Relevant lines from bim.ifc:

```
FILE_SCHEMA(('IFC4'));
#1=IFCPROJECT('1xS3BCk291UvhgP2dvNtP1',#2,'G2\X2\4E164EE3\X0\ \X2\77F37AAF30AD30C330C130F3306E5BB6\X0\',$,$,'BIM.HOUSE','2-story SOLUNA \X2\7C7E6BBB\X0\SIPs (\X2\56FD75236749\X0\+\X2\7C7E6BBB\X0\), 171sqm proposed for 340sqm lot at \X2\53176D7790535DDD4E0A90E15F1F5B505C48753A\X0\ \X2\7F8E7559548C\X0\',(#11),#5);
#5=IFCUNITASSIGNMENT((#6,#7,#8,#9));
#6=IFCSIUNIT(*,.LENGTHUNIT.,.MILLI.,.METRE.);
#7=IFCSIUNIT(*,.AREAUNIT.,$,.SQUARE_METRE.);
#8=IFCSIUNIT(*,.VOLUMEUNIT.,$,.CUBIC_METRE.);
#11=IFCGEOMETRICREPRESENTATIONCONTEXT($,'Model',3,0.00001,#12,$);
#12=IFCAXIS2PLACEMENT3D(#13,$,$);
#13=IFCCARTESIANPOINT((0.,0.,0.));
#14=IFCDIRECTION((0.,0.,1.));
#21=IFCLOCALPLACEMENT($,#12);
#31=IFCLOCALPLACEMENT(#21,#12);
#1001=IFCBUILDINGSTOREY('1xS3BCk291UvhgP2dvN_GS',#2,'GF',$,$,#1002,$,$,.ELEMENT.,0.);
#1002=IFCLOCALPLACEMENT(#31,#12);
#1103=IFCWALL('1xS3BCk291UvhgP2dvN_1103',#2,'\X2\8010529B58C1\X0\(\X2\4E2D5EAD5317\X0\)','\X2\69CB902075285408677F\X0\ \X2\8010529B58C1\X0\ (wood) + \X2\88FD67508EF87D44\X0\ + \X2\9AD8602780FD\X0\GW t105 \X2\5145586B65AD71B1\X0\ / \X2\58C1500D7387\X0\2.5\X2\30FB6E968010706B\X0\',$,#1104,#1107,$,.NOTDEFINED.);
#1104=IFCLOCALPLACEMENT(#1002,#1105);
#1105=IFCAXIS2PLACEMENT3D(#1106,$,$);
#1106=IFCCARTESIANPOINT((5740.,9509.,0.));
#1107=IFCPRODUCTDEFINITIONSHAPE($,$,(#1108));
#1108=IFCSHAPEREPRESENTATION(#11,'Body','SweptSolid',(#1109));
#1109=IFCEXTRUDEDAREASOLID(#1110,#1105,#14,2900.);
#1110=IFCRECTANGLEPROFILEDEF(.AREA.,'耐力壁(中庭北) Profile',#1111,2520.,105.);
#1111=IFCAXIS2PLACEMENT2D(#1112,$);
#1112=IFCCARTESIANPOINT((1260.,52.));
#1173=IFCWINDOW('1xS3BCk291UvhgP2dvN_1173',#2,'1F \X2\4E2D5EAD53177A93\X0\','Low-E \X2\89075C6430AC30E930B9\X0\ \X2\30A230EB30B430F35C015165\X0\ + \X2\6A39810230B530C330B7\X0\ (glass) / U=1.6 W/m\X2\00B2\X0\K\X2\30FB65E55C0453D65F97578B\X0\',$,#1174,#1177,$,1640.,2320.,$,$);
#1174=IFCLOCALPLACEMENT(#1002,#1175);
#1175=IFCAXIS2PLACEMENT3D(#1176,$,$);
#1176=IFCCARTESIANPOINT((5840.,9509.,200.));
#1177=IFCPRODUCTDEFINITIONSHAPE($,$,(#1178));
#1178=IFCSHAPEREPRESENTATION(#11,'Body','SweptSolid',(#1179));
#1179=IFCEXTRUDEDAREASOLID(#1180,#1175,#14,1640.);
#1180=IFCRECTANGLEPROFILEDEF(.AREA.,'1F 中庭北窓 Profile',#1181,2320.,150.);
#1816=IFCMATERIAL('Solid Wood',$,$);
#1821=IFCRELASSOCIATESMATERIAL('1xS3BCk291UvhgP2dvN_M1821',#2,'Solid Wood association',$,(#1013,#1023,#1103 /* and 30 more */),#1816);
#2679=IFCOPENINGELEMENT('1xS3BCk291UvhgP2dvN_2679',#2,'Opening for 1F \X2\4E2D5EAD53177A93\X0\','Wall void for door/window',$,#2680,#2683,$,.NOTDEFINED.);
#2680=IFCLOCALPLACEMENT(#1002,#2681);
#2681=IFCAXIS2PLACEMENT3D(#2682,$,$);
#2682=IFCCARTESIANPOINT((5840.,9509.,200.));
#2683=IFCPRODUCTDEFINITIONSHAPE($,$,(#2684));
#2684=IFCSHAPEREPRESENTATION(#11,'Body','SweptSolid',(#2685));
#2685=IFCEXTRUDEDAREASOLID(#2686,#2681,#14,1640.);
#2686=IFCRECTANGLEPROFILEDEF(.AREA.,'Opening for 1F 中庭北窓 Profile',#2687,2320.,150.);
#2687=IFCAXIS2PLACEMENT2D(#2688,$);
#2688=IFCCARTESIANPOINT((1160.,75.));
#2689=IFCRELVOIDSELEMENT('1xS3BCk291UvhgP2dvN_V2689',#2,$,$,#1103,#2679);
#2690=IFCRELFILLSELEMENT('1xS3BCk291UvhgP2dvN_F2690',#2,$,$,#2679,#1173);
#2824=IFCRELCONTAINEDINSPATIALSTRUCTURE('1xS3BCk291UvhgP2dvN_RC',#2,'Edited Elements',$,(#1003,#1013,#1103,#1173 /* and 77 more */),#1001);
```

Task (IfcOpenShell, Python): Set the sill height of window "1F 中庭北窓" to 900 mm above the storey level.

```python
import numpy as np
import ifcopenshell
import ifcopenshell.api.geometry
import ifcopenshell.geom
import ifcopenshell.util.element
import ifcopenshell.util.placement
import ifcopenshell.util.shape
import ifcopenshell.util.unit

model = ifcopenshell.open("bim.ifc")
unit_scale = ifcopenshell.util.unit.calculate_unit_scale(model)

window = model.by_id(1173)
opening = window.FillsVoids[0].RelatingOpeningElement
storey = ifcopenshell.util.element.get_container(window, ifc_class="IfcBuildingStorey")
level = ifcopenshell.util.placement.get_local_placement(storey.ObjectPlacement)[2, 3]

# The opening's origin need not be at the sill, so measure its lowest point.
shape = ifcopenshell.geom.create_shape(ifcopenshell.geom.settings(), opening)
bottom = ifcopenshell.util.shape.get_shape_bottom_elevation(shape, shape.geometry) / unit_scale
dz = level + 0.9 / unit_scale - bottom

shift = np.array([0.0, 0.0, dz])
# The window is not placed relative to its opening, so move both.
for product in (opening, window):
    matrix = ifcopenshell.util.placement.get_local_placement(product.ObjectPlacement)
    matrix[:3, 3] += shift
    ifcopenshell.api.geometry.edit_object_placement(model, product=product, matrix=matrix, is_si=False)

print(f"moved by {dz * unit_scale:+.3f} m")

model.write("bim_edited.ifc")
```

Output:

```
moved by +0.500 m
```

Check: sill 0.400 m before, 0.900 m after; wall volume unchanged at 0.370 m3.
